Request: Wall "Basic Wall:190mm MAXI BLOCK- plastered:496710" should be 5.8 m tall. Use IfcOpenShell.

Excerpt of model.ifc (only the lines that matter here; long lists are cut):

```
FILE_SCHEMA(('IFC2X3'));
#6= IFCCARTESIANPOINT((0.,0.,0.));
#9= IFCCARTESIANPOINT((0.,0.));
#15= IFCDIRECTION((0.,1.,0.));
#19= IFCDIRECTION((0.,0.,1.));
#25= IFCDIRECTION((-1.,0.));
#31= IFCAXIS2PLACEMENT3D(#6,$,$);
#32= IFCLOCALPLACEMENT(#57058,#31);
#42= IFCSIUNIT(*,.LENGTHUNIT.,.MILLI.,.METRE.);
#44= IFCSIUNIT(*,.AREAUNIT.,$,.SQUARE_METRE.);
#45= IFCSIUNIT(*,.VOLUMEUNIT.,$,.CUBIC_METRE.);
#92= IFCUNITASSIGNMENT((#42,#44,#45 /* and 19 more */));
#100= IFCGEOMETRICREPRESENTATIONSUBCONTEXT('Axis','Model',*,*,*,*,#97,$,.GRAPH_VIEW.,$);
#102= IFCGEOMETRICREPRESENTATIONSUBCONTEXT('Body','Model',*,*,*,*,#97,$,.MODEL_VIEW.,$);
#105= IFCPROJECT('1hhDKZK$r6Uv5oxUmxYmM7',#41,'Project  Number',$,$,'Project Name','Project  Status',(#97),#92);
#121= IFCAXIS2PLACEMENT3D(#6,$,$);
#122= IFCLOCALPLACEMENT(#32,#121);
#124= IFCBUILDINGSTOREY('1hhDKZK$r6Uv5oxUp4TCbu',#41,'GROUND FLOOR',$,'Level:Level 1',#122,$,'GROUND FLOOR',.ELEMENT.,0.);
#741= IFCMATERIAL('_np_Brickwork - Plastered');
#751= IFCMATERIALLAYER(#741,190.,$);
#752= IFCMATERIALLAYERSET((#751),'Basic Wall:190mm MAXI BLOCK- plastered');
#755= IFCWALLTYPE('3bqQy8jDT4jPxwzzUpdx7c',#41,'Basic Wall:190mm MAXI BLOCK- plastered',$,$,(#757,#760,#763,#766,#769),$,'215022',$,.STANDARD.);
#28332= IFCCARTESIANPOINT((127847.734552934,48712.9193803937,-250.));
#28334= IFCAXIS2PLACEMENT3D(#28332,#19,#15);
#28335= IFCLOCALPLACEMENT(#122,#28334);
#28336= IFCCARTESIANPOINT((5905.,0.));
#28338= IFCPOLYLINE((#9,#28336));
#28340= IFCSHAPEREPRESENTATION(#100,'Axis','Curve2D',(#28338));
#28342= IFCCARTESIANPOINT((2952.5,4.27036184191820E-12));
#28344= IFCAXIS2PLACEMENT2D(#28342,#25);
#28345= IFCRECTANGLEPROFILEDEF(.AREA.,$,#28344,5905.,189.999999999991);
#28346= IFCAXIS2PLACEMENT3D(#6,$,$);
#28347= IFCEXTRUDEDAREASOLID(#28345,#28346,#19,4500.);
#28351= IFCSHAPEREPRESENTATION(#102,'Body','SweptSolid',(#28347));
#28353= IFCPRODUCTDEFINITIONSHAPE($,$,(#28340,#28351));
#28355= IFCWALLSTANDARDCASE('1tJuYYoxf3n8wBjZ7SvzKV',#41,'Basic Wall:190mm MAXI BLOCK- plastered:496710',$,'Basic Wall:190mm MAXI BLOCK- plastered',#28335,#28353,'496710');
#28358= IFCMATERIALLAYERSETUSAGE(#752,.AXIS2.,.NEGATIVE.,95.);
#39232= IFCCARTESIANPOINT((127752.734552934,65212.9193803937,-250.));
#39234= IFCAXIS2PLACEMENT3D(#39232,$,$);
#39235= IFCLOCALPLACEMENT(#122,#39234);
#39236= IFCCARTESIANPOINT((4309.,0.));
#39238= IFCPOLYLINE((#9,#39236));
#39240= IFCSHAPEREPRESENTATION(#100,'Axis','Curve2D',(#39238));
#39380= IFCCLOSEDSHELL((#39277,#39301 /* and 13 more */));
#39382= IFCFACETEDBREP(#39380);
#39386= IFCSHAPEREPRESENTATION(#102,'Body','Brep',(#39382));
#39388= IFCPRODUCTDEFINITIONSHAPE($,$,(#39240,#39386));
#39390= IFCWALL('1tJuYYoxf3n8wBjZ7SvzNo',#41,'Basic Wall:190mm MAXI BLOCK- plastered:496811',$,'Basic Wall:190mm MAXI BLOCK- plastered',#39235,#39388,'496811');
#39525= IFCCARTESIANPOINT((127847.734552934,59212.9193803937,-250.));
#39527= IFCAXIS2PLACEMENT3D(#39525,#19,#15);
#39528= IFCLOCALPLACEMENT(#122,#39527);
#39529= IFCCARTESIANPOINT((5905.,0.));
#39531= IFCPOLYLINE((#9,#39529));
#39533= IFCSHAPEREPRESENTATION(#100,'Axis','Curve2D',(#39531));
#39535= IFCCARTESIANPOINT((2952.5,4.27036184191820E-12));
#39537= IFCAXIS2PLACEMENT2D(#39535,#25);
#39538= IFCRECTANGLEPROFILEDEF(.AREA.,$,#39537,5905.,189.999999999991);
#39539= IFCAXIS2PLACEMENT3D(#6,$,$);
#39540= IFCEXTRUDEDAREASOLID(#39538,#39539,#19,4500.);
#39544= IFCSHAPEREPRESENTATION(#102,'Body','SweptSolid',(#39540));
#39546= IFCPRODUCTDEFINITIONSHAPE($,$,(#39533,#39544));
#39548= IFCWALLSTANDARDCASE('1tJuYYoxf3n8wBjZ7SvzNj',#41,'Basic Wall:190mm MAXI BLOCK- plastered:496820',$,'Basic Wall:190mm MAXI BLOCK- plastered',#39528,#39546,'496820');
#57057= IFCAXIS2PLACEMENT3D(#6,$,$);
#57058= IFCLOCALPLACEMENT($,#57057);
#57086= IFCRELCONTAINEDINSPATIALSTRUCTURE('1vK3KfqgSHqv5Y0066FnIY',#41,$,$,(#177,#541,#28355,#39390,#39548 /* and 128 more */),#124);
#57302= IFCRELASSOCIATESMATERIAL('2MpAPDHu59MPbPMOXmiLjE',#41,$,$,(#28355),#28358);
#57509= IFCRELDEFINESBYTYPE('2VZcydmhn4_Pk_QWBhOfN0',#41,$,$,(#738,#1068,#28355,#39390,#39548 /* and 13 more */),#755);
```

```python
import ifcopenshell
import ifcopenshell.geom
import ifcopenshell.util.representation
import ifcopenshell.util.shape
import ifcopenshell.util.unit

model = ifcopenshell.open("model.ifc")
unit_scale = ifcopenshell.util.unit.calculate_unit_scale(model)
settings = ifcopenshell.geom.settings()


def volume(element):
    """Net volume in cubic metres, openings subtracted."""
    shape = ifcopenshell.geom.create_shape(settings, element)
    return ifcopenshell.util.shape.get_volume(shape.geometry)


wall = model.by_id(28355)
before = volume(wall)

body = ifcopenshell.util.representation.get_representation(wall, "Model", "Body")
solid = body.Items[0]
old_height = solid.Depth
solid.Depth = 5.8 / unit_scale
after = volume(wall)

print(f"height {old_height:g} -> {solid.Depth:g}, volume {before:.3f} -> {after:.3f} m3")

model.write("model_updated.ifc")
```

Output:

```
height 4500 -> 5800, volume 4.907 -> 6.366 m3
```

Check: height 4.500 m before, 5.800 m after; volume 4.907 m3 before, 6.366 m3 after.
